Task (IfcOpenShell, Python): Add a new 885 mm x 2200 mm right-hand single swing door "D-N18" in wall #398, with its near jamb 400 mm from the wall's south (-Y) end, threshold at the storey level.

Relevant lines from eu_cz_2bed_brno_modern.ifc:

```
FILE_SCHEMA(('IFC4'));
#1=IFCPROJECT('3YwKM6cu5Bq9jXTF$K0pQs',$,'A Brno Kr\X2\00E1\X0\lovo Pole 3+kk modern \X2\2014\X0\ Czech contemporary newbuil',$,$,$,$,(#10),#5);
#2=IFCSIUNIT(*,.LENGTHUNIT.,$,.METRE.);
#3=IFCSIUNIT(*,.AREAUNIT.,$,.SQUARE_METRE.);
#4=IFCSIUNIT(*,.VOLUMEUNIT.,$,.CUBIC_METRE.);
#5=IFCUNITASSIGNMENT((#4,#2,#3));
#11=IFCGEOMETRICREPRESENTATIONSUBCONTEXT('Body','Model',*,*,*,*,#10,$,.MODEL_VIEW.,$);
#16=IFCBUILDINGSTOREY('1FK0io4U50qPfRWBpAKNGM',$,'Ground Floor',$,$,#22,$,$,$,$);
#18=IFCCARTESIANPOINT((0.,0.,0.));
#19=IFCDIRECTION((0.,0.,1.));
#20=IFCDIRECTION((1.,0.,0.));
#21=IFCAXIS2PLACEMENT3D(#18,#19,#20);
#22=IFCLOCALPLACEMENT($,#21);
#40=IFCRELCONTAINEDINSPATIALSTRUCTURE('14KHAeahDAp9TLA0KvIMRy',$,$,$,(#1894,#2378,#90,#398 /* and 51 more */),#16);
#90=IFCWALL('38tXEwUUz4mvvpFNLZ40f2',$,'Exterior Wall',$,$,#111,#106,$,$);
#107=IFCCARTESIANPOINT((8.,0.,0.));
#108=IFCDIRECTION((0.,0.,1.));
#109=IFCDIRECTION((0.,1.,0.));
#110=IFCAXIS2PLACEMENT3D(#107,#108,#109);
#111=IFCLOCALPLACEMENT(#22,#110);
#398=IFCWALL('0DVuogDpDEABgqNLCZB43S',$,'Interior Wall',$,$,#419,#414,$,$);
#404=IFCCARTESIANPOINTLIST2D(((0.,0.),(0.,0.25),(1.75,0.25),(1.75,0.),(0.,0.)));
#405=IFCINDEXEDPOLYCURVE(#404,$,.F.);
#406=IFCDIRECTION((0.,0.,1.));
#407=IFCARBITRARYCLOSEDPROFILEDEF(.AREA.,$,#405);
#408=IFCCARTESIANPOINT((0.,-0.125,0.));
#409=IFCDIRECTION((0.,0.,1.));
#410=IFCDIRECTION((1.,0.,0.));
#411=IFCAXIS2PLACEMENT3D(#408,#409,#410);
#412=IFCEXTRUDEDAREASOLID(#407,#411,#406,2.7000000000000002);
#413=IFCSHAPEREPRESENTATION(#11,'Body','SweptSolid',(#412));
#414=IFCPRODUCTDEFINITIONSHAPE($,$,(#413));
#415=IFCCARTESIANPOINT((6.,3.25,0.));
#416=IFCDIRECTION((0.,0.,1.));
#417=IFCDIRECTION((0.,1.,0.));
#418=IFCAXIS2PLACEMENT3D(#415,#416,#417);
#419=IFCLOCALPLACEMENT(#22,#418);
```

```python
import numpy as np
import ifcopenshell
import ifcopenshell.api.feature
import ifcopenshell.api.geometry
import ifcopenshell.api.root
import ifcopenshell.api.spatial
import ifcopenshell.geom
import ifcopenshell.util.element
import ifcopenshell.util.placement
import ifcopenshell.util.representation
import ifcopenshell.util.shape
import ifcopenshell.util.unit

model = ifcopenshell.open("eu_cz_2bed_brno_modern.ifc")
unit_scale = ifcopenshell.util.unit.calculate_unit_scale(model)
settings = ifcopenshell.geom.settings()


def volume(element):
    """Net volume in cubic metres, openings subtracted."""
    shape = ifcopenshell.geom.create_shape(settings, element)
    return ifcopenshell.util.shape.get_volume(shape.geometry)


wall = model.by_id(398)
storey = ifcopenshell.util.element.get_container(wall, ifc_class="IfcBuildingStorey")
context = ifcopenshell.util.representation.get_context(model, "Model", "Body", "MODEL_VIEW")
before = volume(wall)

width, height, from_end, sill = 0.885, 2.2, 0.4, 0.0  # metres

# The wall runs along its own X axis, and the end named is its -X end.
wall_shape = ifcopenshell.geom.create_shape(settings, wall)
x, y, z = ifcopenshell.util.shape.get_vertices(wall_shape.geometry).T
start = x.min() + from_end
face, thickness = float(y.min()), float(y.max() - y.min())
wall_matrix = ifcopenshell.util.placement.get_local_placement(wall.ObjectPlacement)
level = ifcopenshell.util.placement.get_local_placement(storey.ObjectPlacement)[2, 3]


def in_wall(x, y):
    """Placement at x, y metres in the wall's axes, at sill height."""
    matrix = wall_matrix.copy()
    matrix[:, 3] = wall_matrix @ np.array([x / unit_scale, y / unit_scale, 0.0, 1.0])
    matrix[2, 3] = level + sill / unit_scale
    return matrix


# Opening: a box that overshoots both wall faces by 50 mm.
opening = ifcopenshell.api.root.create_entity(model, ifc_class="IfcOpeningElement", predefined_type="OPENING")
box = ifcopenshell.api.geometry.add_wall_representation(
    model, context=context, length=width, height=height, thickness=thickness + 0.1
)
ifcopenshell.api.geometry.assign_representation(model, product=opening, representation=box)
ifcopenshell.api.geometry.edit_object_placement(model, product=opening, matrix=in_wall(start, face - 0.05), is_si=False)
ifcopenshell.api.feature.add_feature(model, feature=opening, element=wall)

door = ifcopenshell.api.root.create_entity(model, ifc_class="IfcDoor", name="D-N18", predefined_type="DOOR")
door.OverallWidth, door.OverallHeight = width / unit_scale, height / unit_scale
door.OperationType = "SINGLE_SWING_RIGHT"
body = ifcopenshell.api.geometry.add_door_representation(
    model,
    context=context,
    overall_width=door.OverallWidth,
    overall_height=door.OverallHeight,
    operation_type="SINGLE_SWING_RIGHT",
    lining_properties={"LiningDepth": thickness / unit_scale, "ThresholdDepth": thickness / unit_scale},
)
ifcopenshell.api.geometry.assign_representation(model, product=door, representation=body)
ifcopenshell.api.spatial.assign_container(model, products=[door], relating_structure=storey)
ifcopenshell.api.feature.add_filling(model, opening=opening, element=door)

# The lining spans the wall, so the door starts at the wall face.
ifcopenshell.api.geometry.edit_object_placement(model, product=door, matrix=in_wall(start, face), is_si=False)

after = volume(wall)

print(f"wall volume {before:.3f} -> {after:.3f} m3")

model.write("eu_cz_2bed_brno_modern-out.ifc")
```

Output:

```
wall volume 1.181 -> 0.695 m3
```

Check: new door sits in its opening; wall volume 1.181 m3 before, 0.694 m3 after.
